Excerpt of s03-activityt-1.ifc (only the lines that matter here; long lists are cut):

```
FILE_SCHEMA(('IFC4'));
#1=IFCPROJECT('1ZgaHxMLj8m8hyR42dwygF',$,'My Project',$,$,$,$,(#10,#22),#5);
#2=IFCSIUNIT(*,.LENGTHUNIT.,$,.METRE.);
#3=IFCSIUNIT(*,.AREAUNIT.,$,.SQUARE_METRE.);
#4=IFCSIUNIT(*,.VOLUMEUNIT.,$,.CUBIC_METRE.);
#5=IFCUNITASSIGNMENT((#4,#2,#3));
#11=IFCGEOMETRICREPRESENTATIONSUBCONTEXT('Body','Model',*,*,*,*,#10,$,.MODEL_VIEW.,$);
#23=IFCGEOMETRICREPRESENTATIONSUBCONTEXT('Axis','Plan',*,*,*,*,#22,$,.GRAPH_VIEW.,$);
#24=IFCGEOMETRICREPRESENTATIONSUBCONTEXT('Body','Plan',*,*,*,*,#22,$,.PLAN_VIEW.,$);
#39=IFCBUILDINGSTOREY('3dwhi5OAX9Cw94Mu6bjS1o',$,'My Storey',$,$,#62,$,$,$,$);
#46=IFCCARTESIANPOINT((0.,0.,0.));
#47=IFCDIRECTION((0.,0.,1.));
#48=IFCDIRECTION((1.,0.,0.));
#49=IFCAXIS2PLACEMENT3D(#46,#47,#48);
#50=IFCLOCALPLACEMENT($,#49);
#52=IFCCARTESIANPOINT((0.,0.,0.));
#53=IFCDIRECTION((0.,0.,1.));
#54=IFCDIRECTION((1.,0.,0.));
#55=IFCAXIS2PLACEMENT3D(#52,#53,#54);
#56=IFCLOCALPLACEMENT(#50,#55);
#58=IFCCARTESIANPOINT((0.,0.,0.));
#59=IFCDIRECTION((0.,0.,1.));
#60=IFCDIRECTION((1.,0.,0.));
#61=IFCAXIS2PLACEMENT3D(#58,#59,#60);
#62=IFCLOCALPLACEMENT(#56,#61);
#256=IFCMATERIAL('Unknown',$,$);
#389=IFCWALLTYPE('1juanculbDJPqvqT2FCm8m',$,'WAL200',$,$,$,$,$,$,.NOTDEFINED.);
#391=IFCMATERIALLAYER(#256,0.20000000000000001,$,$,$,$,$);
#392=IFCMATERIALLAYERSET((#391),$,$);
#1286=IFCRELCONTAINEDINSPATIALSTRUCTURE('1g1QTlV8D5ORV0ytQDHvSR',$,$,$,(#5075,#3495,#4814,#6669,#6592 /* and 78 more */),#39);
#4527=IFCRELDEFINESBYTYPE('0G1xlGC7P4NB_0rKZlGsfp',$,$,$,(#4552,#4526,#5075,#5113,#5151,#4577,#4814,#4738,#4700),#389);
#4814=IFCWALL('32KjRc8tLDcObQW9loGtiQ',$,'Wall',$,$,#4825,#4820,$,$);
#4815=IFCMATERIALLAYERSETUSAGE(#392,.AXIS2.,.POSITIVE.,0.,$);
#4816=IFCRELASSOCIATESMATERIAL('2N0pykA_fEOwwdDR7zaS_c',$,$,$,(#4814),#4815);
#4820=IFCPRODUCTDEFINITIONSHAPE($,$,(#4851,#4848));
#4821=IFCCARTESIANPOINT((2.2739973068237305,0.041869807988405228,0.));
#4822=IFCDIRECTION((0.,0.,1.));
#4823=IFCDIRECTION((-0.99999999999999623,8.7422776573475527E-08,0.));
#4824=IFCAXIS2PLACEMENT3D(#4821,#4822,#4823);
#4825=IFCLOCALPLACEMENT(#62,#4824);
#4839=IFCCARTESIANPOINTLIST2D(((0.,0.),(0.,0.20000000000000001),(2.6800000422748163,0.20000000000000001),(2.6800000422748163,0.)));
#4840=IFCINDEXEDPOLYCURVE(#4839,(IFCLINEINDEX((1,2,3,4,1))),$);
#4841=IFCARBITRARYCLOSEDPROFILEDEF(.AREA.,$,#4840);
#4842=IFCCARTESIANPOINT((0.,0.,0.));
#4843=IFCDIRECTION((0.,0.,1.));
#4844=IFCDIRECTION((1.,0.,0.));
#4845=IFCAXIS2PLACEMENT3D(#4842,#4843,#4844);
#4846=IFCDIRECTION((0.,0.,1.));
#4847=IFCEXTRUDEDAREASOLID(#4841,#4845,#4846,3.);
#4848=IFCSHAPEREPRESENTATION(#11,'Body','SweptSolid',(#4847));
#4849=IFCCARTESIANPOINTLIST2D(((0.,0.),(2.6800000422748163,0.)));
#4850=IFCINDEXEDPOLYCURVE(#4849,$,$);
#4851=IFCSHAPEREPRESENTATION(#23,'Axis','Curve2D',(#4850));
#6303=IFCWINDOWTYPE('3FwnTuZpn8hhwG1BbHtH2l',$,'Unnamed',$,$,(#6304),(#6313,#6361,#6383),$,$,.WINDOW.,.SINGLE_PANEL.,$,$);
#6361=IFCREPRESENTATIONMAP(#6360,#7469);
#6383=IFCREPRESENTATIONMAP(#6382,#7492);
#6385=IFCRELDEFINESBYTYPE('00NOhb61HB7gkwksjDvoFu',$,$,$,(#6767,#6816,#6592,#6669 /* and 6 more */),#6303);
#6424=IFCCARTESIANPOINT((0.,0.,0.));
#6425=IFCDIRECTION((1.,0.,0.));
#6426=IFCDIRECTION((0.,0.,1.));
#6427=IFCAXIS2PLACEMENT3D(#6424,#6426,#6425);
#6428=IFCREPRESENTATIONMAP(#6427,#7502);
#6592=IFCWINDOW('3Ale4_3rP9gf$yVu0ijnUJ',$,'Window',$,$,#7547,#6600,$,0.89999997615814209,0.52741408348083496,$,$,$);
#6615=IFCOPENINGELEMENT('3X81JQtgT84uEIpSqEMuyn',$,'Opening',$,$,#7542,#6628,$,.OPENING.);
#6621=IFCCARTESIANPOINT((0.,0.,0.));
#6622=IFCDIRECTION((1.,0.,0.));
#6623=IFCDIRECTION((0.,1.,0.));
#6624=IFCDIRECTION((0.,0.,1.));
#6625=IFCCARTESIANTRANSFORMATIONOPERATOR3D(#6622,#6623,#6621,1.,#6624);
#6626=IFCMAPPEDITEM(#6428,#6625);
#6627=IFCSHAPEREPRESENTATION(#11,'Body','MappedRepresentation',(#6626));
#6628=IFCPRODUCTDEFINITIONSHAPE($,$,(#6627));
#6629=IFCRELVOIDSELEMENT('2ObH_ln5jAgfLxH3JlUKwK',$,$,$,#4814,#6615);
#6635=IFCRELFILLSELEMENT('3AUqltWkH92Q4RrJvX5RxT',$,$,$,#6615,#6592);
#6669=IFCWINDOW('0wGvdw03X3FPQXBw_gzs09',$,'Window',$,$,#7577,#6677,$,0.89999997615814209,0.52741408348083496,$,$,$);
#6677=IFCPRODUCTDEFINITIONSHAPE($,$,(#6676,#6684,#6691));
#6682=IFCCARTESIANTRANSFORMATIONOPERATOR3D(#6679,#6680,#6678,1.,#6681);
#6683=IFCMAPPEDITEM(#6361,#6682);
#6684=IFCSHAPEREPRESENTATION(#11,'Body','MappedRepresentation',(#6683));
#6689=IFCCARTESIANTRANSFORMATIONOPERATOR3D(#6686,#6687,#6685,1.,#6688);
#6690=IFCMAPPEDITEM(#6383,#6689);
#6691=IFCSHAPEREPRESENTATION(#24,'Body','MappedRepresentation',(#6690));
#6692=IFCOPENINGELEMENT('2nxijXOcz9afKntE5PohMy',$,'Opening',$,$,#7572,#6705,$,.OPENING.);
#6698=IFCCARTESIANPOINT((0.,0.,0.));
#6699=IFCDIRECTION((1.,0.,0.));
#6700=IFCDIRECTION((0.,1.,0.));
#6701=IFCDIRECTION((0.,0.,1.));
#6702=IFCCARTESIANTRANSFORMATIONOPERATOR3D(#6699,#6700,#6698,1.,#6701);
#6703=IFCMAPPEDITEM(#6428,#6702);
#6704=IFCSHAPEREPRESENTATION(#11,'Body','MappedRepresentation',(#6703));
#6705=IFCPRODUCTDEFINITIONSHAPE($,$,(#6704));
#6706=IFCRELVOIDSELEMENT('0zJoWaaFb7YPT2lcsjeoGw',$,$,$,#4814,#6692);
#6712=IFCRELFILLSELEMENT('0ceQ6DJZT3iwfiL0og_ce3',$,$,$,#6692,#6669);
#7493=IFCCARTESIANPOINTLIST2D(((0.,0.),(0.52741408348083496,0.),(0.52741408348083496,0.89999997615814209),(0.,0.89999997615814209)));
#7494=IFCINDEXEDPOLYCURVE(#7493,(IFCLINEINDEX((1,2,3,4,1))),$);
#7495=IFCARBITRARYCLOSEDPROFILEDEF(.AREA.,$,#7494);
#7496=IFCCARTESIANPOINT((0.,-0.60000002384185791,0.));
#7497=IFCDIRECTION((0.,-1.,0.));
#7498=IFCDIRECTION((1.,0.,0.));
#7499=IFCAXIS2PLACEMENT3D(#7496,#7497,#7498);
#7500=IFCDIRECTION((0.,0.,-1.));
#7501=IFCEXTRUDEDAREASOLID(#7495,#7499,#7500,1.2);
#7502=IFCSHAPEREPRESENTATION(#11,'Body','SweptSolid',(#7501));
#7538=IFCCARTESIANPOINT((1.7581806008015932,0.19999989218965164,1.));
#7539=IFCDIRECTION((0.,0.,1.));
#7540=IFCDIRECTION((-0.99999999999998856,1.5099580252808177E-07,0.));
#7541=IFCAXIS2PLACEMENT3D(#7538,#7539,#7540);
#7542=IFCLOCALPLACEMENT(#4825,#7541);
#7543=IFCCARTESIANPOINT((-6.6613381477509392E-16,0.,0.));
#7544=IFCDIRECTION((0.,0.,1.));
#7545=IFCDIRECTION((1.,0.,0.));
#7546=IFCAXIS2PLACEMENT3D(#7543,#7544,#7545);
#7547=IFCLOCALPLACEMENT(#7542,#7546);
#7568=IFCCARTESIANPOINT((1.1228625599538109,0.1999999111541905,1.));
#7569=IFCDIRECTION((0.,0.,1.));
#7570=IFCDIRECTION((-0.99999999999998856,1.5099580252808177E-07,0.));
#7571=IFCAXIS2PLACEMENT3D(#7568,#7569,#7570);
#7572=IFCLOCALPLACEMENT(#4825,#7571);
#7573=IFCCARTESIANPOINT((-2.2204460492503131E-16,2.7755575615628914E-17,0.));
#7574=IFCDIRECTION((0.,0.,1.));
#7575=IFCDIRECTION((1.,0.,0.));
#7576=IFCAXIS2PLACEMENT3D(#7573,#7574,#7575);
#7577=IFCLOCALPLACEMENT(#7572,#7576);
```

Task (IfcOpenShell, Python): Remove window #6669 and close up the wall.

```python
import ifcopenshell
import ifcopenshell.api.feature
import ifcopenshell.api.root
import ifcopenshell.geom
import ifcopenshell.util.shape

model = ifcopenshell.open("s03-activityt-1.ifc")
settings = ifcopenshell.geom.settings()


def volume(element):
    """Net volume in cubic metres, openings subtracted."""
    shape = ifcopenshell.geom.create_shape(settings, element)
    return ifcopenshell.util.shape.get_volume(shape.geometry)


window = model.by_id(6669)
opening = window.FillsVoids[0].RelatingOpeningElement
wall = opening.VoidsElements[0].RelatingBuildingElement
before = volume(wall)

ifcopenshell.api.root.remove_product(model, product=window)
ifcopenshell.api.feature.remove_feature(model, feature=opening)

after = volume(wall)

print(f"wall volume {before:.3f} -> {after:.3f} m3")

model.write("s03-activityt-1-out.ifc")
```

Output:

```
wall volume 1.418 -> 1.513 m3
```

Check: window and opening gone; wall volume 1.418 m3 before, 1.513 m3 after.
